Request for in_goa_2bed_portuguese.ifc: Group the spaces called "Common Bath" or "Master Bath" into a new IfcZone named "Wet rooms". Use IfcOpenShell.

First a look at what the model holds.

```python
import ifcopenshell

model = ifcopenshell.open("in_goa_2bed_portuguese.ifc")
print(model.schema)
seen = {}
for space in model.by_type("IfcSpace"):
    seen[space.LongName] = seen.get(space.LongName, 0) + 1
for name, count in sorted(seen.items(), key=str):
    print(count, "x", name)
print("zones:", [z.Name for z in model.by_type("IfcZone")][:20])
```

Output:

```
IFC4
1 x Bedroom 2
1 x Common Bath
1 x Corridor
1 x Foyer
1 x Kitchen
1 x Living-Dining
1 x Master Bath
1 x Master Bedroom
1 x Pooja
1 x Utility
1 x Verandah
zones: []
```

```python
import ifcopenshell
import ifcopenshell.api.group
import ifcopenshell.api.root

model = ifcopenshell.open("in_goa_2bed_portuguese.ifc")

names = {"Common Bath", "Master Bath"}
spaces = [s for s in model.by_type("IfcSpace") if s.LongName in names]

zone = ifcopenshell.api.root.create_entity(model, ifc_class="IfcZone", name="Wet rooms")
ifcopenshell.api.group.assign_group(model, products=spaces, group=zone)
print(len(spaces), "spaces in", zone.Name)

model.write("in_goa_2bed_portuguese_v2.ifc")
```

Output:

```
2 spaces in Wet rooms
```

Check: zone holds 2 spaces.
